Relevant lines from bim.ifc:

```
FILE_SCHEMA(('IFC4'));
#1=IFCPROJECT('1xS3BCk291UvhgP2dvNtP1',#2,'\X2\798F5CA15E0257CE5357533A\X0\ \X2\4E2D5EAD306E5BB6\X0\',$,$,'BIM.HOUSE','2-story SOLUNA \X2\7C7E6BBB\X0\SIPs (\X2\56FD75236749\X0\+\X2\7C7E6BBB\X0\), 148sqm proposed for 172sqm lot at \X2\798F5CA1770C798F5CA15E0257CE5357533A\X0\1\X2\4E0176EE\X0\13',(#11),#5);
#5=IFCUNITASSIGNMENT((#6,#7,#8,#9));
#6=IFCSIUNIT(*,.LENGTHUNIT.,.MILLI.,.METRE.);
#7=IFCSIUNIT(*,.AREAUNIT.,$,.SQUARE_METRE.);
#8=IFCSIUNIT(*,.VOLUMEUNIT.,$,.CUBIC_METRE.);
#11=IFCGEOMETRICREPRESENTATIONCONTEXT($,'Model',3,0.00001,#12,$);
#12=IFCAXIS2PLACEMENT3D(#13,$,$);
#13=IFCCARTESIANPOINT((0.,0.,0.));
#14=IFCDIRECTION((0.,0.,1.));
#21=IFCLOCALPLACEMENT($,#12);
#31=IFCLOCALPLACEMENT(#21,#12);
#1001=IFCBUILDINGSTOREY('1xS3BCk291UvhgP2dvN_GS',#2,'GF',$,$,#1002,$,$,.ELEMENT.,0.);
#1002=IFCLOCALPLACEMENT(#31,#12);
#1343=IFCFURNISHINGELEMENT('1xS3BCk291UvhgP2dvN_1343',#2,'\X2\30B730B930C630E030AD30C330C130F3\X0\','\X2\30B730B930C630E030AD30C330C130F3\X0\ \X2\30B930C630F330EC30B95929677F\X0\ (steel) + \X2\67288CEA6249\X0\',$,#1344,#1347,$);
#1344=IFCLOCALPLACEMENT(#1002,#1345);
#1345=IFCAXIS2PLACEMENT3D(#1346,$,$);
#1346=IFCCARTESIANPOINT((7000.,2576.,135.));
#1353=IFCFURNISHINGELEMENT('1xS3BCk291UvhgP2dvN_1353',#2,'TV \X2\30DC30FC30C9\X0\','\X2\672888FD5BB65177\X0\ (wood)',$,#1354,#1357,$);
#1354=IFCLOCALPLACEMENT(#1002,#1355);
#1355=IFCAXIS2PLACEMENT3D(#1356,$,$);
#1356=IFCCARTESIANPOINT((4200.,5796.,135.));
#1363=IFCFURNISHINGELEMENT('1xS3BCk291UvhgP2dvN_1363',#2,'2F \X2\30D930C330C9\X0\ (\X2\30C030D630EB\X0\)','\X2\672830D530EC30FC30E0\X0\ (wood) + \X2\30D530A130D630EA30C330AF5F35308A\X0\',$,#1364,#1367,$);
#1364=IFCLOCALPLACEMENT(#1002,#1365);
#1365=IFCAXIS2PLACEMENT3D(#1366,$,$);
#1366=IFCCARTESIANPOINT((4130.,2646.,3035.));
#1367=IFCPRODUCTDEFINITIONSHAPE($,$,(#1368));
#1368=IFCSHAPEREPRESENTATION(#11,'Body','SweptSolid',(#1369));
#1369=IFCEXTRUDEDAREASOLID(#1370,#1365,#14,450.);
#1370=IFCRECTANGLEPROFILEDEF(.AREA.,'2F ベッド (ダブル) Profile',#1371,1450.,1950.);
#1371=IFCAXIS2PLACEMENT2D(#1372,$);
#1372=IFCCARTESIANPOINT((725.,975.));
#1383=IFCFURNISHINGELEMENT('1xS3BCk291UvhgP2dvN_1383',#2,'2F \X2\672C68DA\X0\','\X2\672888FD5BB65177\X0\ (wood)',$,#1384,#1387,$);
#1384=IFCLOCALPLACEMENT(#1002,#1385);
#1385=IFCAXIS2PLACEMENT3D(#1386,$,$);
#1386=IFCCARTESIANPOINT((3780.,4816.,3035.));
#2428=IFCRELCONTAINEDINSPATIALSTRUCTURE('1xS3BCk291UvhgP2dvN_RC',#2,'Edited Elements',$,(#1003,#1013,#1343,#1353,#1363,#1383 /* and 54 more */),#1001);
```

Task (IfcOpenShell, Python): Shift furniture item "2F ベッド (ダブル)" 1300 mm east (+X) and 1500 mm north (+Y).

```python
import ifcopenshell
import ifcopenshell.api.geometry
import ifcopenshell.util.placement

model = ifcopenshell.open("bim.ifc")

item = model.by_guid("1xS3BCk291UvhgP2dvN_1363")
matrix = ifcopenshell.util.placement.get_local_placement(item.ObjectPlacement)
matrix[0, 3] += 1300.0
matrix[1, 3] += 1500.0
ifcopenshell.api.geometry.edit_object_placement(model, product=item, matrix=matrix, is_si=False)

print(ifcopenshell.util.placement.get_local_placement(item.ObjectPlacement).round(3) + 0.0)

model.write("bim_rev.ifc")
```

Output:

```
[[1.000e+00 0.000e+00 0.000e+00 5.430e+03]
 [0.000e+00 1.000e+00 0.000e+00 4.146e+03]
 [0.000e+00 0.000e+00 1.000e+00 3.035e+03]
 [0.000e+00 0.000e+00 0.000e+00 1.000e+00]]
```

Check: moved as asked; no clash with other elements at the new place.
